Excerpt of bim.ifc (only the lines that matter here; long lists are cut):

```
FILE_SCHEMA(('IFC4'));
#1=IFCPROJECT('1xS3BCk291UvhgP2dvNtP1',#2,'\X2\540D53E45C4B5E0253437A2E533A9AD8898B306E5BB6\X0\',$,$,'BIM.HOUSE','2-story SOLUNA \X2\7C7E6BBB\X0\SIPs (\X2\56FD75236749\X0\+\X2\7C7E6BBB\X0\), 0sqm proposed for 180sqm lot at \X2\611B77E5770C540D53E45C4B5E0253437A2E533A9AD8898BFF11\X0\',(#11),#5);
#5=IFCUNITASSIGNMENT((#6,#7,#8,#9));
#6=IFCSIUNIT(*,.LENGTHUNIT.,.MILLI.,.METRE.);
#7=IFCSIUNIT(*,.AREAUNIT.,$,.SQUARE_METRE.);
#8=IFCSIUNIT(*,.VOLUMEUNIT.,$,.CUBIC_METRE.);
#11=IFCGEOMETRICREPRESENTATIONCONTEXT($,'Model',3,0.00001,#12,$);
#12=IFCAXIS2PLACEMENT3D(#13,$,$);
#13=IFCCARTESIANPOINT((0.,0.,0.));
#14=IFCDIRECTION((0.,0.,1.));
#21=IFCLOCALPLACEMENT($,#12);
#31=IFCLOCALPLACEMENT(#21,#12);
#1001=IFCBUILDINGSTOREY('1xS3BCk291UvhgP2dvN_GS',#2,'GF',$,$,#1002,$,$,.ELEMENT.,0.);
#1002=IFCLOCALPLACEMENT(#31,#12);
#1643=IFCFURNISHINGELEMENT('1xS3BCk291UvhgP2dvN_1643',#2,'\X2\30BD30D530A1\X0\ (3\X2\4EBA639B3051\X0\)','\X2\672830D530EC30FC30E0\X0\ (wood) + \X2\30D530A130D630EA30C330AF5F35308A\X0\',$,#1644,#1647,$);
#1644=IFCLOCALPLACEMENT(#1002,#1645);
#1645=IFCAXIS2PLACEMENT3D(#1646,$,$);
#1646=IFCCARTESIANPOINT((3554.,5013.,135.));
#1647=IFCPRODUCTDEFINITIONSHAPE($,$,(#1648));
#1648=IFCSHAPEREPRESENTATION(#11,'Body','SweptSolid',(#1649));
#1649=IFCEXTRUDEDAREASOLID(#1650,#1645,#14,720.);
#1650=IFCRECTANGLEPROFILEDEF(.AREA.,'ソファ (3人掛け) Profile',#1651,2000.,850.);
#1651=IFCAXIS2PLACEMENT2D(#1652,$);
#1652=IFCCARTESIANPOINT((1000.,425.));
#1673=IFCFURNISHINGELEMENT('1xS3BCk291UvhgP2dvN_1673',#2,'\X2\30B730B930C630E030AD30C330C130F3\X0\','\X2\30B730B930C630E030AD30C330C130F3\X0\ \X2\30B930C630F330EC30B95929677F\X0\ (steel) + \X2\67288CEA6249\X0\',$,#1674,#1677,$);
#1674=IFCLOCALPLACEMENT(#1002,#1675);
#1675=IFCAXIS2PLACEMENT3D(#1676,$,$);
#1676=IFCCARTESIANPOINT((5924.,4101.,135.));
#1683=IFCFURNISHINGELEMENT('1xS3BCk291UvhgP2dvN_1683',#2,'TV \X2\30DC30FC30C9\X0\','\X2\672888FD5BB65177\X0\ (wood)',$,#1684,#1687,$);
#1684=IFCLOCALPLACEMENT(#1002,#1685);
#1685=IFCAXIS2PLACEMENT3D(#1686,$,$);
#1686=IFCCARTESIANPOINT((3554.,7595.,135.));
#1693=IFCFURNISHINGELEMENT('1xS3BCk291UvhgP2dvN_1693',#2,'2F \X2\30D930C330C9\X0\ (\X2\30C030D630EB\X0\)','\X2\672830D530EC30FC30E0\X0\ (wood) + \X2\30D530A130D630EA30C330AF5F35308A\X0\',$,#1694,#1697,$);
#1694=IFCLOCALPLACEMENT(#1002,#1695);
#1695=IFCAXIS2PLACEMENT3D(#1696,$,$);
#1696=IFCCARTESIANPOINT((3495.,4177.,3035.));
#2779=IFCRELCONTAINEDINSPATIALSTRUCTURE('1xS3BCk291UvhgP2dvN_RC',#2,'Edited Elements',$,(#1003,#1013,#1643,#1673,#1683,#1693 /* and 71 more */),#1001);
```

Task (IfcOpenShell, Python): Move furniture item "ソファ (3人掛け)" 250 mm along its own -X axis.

```python
import ifcopenshell
import ifcopenshell.api.geometry
import ifcopenshell.util.placement

model = ifcopenshell.open("bim.ifc")

item = model.by_guid("1xS3BCk291UvhgP2dvN_1643")
matrix = ifcopenshell.util.placement.get_local_placement(item.ObjectPlacement)
matrix[:3, 3] -= matrix[:3, 0] * 250.0
ifcopenshell.api.geometry.edit_object_placement(model, product=item, matrix=matrix, is_si=False)

print(ifcopenshell.util.placement.get_local_placement(item.ObjectPlacement).round(3) + 0.0)

model.write("bim_updated.ifc")
```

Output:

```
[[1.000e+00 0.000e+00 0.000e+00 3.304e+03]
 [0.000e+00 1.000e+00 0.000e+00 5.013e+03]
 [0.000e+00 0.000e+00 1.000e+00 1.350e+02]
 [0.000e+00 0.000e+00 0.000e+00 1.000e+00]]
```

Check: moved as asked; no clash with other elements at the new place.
